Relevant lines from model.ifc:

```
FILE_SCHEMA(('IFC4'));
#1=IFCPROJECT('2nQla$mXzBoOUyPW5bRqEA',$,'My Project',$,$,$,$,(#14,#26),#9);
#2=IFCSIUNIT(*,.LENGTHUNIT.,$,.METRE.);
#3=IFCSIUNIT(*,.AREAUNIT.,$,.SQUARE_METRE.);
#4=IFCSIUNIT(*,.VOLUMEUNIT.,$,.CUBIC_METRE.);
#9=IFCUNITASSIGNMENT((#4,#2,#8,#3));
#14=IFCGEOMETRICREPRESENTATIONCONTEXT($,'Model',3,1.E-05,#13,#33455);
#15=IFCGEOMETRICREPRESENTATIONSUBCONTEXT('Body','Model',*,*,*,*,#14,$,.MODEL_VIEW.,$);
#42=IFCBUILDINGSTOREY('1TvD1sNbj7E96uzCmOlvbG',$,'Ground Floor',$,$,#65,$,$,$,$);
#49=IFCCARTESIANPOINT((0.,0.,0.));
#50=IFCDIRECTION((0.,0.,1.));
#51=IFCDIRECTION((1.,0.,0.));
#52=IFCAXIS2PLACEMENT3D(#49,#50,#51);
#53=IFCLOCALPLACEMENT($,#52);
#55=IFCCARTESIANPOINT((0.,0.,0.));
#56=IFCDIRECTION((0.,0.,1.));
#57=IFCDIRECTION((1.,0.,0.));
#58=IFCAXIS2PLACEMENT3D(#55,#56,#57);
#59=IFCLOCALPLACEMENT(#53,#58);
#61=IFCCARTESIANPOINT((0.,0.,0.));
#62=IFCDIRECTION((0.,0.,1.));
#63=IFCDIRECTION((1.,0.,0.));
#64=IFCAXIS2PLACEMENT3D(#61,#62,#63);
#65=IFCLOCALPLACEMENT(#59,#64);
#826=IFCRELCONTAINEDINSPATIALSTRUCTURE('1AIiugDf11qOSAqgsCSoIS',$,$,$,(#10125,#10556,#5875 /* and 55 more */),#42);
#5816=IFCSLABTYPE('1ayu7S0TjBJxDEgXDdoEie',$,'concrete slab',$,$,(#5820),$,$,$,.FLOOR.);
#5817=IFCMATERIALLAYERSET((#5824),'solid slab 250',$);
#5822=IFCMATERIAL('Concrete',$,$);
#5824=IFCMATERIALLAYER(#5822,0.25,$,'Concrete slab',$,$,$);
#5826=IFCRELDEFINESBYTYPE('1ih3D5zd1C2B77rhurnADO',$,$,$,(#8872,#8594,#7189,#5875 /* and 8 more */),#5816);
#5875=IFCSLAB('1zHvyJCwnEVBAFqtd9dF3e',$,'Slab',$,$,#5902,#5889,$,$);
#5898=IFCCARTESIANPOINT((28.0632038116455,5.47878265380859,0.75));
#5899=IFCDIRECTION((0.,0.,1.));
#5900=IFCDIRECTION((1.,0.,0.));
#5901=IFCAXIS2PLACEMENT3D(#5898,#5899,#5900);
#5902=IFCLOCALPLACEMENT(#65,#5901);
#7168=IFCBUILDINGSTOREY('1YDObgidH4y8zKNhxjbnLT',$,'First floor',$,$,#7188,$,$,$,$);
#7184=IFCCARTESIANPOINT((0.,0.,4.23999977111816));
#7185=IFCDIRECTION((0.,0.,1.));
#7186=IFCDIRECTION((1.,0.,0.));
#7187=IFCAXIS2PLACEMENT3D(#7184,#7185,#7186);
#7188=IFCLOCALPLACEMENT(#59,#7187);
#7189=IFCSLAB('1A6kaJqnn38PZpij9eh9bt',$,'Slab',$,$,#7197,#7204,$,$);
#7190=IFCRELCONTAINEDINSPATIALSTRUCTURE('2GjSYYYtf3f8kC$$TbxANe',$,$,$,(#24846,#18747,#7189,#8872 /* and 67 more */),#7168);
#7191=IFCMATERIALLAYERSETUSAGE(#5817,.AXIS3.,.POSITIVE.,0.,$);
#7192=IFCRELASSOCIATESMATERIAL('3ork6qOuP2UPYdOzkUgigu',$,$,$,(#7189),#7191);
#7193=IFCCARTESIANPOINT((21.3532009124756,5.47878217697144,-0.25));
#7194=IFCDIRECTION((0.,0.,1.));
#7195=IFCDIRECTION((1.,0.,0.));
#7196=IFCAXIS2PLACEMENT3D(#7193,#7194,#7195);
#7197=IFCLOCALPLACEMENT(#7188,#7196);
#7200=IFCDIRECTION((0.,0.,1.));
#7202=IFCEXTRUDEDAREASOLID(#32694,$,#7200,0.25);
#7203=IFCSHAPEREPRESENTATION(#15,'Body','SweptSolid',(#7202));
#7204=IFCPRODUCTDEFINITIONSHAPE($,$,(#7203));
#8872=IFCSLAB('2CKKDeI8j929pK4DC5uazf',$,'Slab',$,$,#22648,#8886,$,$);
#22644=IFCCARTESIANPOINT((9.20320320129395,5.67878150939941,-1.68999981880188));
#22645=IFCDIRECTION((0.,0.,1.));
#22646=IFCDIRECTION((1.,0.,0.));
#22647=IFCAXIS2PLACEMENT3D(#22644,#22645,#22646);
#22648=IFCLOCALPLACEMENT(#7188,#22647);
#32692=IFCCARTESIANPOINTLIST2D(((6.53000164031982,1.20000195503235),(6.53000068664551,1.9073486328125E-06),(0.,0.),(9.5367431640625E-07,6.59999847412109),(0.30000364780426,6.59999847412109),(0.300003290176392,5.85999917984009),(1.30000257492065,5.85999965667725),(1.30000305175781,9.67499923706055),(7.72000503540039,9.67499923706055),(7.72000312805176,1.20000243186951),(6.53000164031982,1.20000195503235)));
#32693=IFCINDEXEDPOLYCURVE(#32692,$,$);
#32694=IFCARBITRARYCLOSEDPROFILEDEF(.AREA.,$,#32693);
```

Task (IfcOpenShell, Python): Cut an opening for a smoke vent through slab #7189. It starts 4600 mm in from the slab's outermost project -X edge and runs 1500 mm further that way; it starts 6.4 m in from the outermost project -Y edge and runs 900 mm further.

```python
import numpy as np
import ifcopenshell
import ifcopenshell.api.feature
import ifcopenshell.api.geometry
import ifcopenshell.api.root
import ifcopenshell.geom
import ifcopenshell.util.placement
import ifcopenshell.util.representation
import ifcopenshell.util.shape
import ifcopenshell.util.unit

model = ifcopenshell.open("model.ifc")
unit_scale = ifcopenshell.util.unit.calculate_unit_scale(model)
settings = ifcopenshell.geom.settings()


def volume(element):
    """Net volume in cubic metres, openings subtracted."""
    shape = ifcopenshell.geom.create_shape(settings, element)
    return ifcopenshell.util.shape.get_volume(shape.geometry)


slab = model.by_guid("1A6kaJqnn38PZpij9eh9bt")
before = volume(slab)

# Extent in the slab's own axes, in metres. The edges named are its -X and -Y sides.
slab_shape = ifcopenshell.geom.create_shape(settings, slab)
vertices = ifcopenshell.util.shape.get_vertices(slab_shape.geometry)
x_min, y_min, bottom = vertices.min(axis=0)
top = vertices[:, 2].max()

opening = ifcopenshell.api.root.create_entity(model, ifc_class="IfcOpeningElement", name="Smoke vent opening", predefined_type="OPENING")
context = ifcopenshell.util.representation.get_context(model, "Model", "Body", "MODEL_VIEW")
width, depth = 1.5, 0.9
outline = [(0.0, 0.0), (width, 0.0), (width, depth), (0.0, depth), (0.0, 0.0)]
# Overshoot both faces by 50 mm so the cut is clean.
shape = ifcopenshell.api.geometry.add_slab_representation(
    model, context=context, depth=top - bottom + 0.1, polyline=outline
)
ifcopenshell.api.geometry.assign_representation(model, product=opening, representation=shape)

matrix = ifcopenshell.util.placement.get_local_placement(slab.ObjectPlacement)
matrix[:, 3] = matrix @ np.append(np.array([x_min + 4.6, y_min + 6.4, bottom - 0.05]) / unit_scale, 1.0)
ifcopenshell.api.geometry.edit_object_placement(model, product=opening, matrix=matrix, is_si=False)
ifcopenshell.api.feature.add_feature(model, feature=opening, element=slab)

after = volume(slab)

print(f"slab volume {before:.3f} -> {after:.3f} m3")

model.write("model_rev.ifc")
```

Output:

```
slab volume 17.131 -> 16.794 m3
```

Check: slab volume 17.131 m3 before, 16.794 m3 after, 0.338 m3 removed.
